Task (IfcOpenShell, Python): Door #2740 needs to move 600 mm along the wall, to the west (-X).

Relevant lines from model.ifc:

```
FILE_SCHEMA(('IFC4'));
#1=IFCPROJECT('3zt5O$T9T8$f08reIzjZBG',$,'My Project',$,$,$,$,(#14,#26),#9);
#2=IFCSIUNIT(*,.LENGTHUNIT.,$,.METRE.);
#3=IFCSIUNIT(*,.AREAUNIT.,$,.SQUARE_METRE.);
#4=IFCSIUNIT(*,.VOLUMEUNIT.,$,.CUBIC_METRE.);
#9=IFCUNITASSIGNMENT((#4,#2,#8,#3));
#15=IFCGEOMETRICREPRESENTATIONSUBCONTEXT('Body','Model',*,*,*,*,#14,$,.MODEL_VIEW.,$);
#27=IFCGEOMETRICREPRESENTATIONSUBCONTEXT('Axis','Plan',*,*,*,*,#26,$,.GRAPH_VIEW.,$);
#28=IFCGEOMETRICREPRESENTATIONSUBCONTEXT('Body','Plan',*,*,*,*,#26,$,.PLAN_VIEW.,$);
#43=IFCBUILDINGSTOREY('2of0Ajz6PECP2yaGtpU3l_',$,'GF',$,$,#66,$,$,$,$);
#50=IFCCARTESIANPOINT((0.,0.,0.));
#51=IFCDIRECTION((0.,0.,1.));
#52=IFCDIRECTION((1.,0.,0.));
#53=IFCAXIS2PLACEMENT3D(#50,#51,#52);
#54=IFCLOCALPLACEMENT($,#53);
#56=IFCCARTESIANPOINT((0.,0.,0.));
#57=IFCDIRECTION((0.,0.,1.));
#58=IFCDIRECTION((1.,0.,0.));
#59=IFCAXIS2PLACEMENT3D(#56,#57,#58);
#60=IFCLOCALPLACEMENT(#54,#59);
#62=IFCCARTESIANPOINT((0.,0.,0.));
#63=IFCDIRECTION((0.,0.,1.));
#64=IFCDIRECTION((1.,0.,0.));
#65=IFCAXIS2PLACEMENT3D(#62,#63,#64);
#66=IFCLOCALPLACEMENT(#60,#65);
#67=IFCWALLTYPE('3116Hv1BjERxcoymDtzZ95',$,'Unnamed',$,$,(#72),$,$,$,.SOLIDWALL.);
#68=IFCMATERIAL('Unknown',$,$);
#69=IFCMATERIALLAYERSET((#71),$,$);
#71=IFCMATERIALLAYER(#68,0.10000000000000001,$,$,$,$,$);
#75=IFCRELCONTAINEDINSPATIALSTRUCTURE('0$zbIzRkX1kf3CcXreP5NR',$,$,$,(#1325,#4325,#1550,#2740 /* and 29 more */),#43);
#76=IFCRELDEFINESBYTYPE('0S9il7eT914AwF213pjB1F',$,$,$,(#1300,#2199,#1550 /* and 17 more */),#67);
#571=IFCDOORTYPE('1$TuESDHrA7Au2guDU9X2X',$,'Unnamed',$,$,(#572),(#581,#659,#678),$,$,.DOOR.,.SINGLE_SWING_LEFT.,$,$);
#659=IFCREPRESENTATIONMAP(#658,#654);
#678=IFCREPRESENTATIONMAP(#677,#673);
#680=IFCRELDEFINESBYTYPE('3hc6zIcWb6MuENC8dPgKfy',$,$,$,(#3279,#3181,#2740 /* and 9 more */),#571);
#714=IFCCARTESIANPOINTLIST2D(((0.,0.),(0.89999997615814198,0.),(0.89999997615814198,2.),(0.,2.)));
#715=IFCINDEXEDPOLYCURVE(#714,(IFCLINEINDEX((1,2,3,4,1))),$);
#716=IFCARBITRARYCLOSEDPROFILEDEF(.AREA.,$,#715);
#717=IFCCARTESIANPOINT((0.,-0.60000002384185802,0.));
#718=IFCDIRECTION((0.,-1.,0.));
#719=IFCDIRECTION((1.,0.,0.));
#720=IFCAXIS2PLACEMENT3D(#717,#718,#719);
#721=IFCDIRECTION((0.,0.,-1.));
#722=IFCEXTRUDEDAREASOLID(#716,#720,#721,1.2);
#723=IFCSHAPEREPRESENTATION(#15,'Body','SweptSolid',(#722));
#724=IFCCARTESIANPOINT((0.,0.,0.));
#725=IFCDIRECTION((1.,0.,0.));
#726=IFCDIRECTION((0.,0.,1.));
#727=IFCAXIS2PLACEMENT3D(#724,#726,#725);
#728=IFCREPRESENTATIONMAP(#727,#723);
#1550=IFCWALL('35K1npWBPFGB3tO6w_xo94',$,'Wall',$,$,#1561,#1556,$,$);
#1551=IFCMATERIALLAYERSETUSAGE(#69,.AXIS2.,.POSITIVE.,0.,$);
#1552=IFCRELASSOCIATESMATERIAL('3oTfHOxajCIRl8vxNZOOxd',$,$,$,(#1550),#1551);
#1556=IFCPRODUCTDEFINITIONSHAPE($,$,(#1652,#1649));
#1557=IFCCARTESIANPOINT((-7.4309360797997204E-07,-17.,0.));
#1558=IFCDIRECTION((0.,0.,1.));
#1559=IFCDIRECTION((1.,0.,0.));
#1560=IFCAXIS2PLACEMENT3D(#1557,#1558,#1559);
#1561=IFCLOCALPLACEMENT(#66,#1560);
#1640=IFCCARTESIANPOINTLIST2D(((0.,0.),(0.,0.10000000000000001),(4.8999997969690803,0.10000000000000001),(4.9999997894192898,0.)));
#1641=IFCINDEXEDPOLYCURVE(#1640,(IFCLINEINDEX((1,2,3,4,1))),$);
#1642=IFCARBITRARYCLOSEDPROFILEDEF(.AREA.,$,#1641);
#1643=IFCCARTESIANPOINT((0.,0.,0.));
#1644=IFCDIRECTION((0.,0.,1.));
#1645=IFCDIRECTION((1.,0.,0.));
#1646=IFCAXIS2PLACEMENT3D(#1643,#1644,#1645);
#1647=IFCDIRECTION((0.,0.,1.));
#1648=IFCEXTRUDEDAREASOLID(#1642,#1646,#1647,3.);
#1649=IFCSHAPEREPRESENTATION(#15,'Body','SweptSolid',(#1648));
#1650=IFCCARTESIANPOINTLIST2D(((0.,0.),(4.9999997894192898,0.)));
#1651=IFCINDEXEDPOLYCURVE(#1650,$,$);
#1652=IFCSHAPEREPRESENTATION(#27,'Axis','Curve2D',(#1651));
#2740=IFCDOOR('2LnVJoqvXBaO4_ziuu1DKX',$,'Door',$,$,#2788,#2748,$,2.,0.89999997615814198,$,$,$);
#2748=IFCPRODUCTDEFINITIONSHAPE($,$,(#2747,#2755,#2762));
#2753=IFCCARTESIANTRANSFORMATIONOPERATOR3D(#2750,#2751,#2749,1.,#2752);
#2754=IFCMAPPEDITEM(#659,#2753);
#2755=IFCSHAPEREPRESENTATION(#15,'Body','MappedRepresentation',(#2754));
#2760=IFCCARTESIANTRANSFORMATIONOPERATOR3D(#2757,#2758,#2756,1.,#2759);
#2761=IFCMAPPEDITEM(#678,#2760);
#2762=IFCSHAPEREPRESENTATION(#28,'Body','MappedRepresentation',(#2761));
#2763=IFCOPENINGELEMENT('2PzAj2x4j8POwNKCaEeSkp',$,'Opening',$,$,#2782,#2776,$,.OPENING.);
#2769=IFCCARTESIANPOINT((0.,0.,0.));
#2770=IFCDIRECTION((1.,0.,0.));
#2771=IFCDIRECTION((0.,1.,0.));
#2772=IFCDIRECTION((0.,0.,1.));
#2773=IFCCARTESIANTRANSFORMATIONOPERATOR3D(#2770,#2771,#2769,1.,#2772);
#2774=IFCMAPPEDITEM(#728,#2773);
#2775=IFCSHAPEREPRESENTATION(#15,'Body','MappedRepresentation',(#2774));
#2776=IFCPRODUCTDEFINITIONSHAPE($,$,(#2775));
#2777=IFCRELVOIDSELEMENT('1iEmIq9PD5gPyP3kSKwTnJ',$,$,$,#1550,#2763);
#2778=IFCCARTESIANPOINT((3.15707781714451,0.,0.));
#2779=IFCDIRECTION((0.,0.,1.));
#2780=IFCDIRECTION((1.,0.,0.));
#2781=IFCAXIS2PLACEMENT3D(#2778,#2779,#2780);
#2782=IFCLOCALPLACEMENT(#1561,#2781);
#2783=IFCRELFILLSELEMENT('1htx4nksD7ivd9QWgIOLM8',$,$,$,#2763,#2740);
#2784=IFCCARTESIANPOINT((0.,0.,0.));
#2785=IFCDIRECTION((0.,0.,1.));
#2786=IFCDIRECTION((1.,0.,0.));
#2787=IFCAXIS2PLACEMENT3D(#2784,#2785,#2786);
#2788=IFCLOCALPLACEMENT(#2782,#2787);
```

```python
import ifcopenshell
import ifcopenshell.api.geometry
import ifcopenshell.util.placement

model = ifcopenshell.open("model.ifc")

door = model.by_id(2740)
opening = door.FillsVoids[0].RelatingOpeningElement
wall = opening.VoidsElements[0].RelatingBuildingElement

wall_matrix = ifcopenshell.util.placement.get_local_placement(wall.ObjectPlacement)
shift = wall_matrix[:3, 0] * -0.6
before = ifcopenshell.util.placement.get_local_placement(door.ObjectPlacement)[:3, 3].copy()

# The door is placed relative to its opening, so it follows when the opening moves.
matrix = ifcopenshell.util.placement.get_local_placement(opening.ObjectPlacement)
matrix[:3, 3] += shift
ifcopenshell.api.geometry.edit_object_placement(
    model, product=opening, matrix=matrix, is_si=False, should_transform_children=True
)

after = ifcopenshell.util.placement.get_local_placement(door.ObjectPlacement)[:3, 3]
print("door moved by", (after - before).round(3) + 0.0)

model.write("model_rev.ifc")
```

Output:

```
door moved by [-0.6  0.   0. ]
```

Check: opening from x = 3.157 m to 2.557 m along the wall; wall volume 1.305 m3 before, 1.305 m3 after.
